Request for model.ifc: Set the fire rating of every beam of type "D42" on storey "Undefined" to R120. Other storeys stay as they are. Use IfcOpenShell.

First a look at what the model holds.

```python
import ifcopenshell
import ifcopenshell.util.element

model = ifcopenshell.open("model.ifc")
print(model.schema)
storey = next(s for s in model.by_type("IfcBuildingStorey") if s.Name == "Undefined")
beams = [e for e in ifcopenshell.util.element.get_decomposition(storey) if e.is_a("IfcBeam")]
seen = {}
for e in beams:
    element_type = ifcopenshell.util.element.get_type(e)
    key = (element_type.Name if element_type != e and element_type else None, ifcopenshell.util.element.get_pset(e, "Pset_BeamCommon", "FireRating"))
    seen[key] = seen.get(key, 0) + 1
for (name, value), count in sorted(seen.items(), key=str):
    print(count, "x", name, "|", value)
```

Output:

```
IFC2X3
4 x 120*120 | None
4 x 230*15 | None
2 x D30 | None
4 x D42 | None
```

```python
import ifcopenshell
import ifcopenshell.api.pset
import ifcopenshell.util.element

model = ifcopenshell.open("model.ifc")

storey = next(s for s in model.by_type("IfcBuildingStorey") if s.Name == "Undefined")
beams = [e for e in ifcopenshell.util.element.get_decomposition(storey) if e.is_a("IfcBeam")]

count = 0
for e in beams:
    element_type = ifcopenshell.util.element.get_type(e)
    if element_type in (None, e) or element_type.Name != "D42":
        continue
    # add_pset returns the element's existing set when there is one.
    pset = ifcopenshell.api.pset.add_pset(model, product=e, name="Pset_BeamCommon")
    ifcopenshell.api.pset.edit_pset(model, pset=pset, properties={"FireRating": "R120"})
    count += 1

print(count, "beams updated")

model.write("model_rev.ifc")
```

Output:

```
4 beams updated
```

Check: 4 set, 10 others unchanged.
